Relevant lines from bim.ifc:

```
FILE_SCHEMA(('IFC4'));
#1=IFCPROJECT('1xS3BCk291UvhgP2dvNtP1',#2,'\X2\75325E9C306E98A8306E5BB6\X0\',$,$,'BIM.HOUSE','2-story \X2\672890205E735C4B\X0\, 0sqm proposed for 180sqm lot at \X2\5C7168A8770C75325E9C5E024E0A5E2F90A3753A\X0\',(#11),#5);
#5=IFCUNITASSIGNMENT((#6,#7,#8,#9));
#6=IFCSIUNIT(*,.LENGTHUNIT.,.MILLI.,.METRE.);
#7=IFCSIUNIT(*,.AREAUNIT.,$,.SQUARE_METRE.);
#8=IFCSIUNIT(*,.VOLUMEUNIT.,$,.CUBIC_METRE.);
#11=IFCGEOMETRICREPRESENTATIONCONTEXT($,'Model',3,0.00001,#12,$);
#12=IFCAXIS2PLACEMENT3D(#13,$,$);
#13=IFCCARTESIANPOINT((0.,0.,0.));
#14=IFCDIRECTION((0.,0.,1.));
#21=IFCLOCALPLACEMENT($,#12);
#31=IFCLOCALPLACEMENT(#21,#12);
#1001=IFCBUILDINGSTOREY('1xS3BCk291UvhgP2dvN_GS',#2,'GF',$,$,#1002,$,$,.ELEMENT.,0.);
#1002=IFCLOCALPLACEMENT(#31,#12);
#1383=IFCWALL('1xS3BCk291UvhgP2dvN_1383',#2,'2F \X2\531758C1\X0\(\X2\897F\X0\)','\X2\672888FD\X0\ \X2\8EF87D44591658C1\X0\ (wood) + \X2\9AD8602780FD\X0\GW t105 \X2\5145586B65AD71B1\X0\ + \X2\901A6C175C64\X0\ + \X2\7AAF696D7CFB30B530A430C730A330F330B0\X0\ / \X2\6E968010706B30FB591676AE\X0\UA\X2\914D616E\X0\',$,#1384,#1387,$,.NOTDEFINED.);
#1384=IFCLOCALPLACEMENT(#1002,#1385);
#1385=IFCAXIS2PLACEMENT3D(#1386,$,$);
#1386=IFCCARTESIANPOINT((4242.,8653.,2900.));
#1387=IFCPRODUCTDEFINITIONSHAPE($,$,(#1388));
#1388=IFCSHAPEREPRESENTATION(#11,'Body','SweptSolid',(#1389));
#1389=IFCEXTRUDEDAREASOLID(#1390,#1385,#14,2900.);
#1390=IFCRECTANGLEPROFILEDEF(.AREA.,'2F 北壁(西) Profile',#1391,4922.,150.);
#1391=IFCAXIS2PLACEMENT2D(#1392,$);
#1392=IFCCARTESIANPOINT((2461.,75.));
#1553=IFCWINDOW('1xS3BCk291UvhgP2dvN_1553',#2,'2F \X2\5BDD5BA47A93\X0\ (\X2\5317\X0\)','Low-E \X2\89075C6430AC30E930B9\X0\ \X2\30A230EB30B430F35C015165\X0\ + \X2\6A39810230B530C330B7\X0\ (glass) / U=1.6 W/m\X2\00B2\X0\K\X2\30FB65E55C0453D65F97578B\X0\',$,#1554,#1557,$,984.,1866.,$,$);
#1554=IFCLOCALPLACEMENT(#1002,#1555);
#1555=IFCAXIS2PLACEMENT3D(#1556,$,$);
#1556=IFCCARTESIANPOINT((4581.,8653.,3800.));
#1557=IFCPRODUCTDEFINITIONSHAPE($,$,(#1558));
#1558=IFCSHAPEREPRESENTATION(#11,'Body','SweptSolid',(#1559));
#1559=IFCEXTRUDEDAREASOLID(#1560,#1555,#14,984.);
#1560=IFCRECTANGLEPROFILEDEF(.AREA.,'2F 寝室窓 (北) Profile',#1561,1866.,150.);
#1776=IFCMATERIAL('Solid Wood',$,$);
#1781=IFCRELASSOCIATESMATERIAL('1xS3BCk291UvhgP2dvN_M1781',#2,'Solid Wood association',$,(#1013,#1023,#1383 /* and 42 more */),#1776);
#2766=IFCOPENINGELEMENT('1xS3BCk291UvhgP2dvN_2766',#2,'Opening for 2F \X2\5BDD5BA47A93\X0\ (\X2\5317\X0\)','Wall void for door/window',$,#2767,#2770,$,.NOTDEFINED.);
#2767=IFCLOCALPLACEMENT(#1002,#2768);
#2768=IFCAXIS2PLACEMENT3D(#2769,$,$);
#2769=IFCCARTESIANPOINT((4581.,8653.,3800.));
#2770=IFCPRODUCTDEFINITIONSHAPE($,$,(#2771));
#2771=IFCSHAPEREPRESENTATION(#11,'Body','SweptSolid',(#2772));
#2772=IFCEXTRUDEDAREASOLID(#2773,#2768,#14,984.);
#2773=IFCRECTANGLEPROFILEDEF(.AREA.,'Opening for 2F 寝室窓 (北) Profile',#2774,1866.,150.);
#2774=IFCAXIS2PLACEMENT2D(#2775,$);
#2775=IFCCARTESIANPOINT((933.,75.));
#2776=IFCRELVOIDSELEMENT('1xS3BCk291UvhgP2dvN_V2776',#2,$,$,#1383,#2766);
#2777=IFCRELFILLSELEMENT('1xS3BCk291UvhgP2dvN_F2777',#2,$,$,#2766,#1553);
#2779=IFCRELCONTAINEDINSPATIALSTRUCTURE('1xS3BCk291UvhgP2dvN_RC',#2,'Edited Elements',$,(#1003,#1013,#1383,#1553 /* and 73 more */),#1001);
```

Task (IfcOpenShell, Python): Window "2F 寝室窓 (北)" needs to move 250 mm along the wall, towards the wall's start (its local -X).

```python
import ifcopenshell
import ifcopenshell.api.geometry
import ifcopenshell.util.placement
import ifcopenshell.util.unit

model = ifcopenshell.open("bim.ifc")
unit_scale = ifcopenshell.util.unit.calculate_unit_scale(model)

window = model.by_guid("1xS3BCk291UvhgP2dvN_1553")
opening = window.FillsVoids[0].RelatingOpeningElement
wall = opening.VoidsElements[0].RelatingBuildingElement

wall_matrix = ifcopenshell.util.placement.get_local_placement(wall.ObjectPlacement)
shift = wall_matrix[:3, 0] * -0.25 / unit_scale
before = ifcopenshell.util.placement.get_local_placement(window.ObjectPlacement)[:3, 3].copy()

# The window is not placed relative to its opening, so move both.
for product in (opening, window):
    matrix = ifcopenshell.util.placement.get_local_placement(product.ObjectPlacement)
    matrix[:3, 3] += shift
    ifcopenshell.api.geometry.edit_object_placement(model, product=product, matrix=matrix, is_si=False)

after = ifcopenshell.util.placement.get_local_placement(window.ObjectPlacement)[:3, 3]
print("window moved by", (after - before).round(3) + 0.0)

model.write("bim_updated.ifc")
```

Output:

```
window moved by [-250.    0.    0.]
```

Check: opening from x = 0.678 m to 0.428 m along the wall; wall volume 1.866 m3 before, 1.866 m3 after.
